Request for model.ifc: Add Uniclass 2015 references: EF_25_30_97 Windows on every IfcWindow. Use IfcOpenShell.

First a look at what the model holds.

```python
import ifcopenshell

model = ifcopenshell.open("model.ifc")
print(model.schema)
print("classifications:", [c.Name for c in model.by_type("IfcClassification")])
for ifc_class in ("IfcDoor", "IfcRoof", "IfcStair", "IfcWall", "IfcWindow"):
    print(ifc_class, len(model.by_type(ifc_class)))
```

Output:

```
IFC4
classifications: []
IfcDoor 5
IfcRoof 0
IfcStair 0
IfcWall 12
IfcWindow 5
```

```python
import ifcopenshell
import ifcopenshell.api.classification

model = ifcopenshell.open("model.ifc")

system = ifcopenshell.api.classification.add_classification(model, classification="Uniclass 2015")

codes = {
    "IfcWindow": ("EF_25_30_97", "Windows"),
}
for ifc_class, (code, name) in codes.items():
    products = model.by_type(ifc_class)
    ifcopenshell.api.classification.add_reference(
        model, products=products, classification=system, identification=code, name=name
    )
    print(code, len(products))

model.write("model_edited.ifc")
```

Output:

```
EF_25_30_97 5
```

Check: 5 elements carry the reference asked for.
